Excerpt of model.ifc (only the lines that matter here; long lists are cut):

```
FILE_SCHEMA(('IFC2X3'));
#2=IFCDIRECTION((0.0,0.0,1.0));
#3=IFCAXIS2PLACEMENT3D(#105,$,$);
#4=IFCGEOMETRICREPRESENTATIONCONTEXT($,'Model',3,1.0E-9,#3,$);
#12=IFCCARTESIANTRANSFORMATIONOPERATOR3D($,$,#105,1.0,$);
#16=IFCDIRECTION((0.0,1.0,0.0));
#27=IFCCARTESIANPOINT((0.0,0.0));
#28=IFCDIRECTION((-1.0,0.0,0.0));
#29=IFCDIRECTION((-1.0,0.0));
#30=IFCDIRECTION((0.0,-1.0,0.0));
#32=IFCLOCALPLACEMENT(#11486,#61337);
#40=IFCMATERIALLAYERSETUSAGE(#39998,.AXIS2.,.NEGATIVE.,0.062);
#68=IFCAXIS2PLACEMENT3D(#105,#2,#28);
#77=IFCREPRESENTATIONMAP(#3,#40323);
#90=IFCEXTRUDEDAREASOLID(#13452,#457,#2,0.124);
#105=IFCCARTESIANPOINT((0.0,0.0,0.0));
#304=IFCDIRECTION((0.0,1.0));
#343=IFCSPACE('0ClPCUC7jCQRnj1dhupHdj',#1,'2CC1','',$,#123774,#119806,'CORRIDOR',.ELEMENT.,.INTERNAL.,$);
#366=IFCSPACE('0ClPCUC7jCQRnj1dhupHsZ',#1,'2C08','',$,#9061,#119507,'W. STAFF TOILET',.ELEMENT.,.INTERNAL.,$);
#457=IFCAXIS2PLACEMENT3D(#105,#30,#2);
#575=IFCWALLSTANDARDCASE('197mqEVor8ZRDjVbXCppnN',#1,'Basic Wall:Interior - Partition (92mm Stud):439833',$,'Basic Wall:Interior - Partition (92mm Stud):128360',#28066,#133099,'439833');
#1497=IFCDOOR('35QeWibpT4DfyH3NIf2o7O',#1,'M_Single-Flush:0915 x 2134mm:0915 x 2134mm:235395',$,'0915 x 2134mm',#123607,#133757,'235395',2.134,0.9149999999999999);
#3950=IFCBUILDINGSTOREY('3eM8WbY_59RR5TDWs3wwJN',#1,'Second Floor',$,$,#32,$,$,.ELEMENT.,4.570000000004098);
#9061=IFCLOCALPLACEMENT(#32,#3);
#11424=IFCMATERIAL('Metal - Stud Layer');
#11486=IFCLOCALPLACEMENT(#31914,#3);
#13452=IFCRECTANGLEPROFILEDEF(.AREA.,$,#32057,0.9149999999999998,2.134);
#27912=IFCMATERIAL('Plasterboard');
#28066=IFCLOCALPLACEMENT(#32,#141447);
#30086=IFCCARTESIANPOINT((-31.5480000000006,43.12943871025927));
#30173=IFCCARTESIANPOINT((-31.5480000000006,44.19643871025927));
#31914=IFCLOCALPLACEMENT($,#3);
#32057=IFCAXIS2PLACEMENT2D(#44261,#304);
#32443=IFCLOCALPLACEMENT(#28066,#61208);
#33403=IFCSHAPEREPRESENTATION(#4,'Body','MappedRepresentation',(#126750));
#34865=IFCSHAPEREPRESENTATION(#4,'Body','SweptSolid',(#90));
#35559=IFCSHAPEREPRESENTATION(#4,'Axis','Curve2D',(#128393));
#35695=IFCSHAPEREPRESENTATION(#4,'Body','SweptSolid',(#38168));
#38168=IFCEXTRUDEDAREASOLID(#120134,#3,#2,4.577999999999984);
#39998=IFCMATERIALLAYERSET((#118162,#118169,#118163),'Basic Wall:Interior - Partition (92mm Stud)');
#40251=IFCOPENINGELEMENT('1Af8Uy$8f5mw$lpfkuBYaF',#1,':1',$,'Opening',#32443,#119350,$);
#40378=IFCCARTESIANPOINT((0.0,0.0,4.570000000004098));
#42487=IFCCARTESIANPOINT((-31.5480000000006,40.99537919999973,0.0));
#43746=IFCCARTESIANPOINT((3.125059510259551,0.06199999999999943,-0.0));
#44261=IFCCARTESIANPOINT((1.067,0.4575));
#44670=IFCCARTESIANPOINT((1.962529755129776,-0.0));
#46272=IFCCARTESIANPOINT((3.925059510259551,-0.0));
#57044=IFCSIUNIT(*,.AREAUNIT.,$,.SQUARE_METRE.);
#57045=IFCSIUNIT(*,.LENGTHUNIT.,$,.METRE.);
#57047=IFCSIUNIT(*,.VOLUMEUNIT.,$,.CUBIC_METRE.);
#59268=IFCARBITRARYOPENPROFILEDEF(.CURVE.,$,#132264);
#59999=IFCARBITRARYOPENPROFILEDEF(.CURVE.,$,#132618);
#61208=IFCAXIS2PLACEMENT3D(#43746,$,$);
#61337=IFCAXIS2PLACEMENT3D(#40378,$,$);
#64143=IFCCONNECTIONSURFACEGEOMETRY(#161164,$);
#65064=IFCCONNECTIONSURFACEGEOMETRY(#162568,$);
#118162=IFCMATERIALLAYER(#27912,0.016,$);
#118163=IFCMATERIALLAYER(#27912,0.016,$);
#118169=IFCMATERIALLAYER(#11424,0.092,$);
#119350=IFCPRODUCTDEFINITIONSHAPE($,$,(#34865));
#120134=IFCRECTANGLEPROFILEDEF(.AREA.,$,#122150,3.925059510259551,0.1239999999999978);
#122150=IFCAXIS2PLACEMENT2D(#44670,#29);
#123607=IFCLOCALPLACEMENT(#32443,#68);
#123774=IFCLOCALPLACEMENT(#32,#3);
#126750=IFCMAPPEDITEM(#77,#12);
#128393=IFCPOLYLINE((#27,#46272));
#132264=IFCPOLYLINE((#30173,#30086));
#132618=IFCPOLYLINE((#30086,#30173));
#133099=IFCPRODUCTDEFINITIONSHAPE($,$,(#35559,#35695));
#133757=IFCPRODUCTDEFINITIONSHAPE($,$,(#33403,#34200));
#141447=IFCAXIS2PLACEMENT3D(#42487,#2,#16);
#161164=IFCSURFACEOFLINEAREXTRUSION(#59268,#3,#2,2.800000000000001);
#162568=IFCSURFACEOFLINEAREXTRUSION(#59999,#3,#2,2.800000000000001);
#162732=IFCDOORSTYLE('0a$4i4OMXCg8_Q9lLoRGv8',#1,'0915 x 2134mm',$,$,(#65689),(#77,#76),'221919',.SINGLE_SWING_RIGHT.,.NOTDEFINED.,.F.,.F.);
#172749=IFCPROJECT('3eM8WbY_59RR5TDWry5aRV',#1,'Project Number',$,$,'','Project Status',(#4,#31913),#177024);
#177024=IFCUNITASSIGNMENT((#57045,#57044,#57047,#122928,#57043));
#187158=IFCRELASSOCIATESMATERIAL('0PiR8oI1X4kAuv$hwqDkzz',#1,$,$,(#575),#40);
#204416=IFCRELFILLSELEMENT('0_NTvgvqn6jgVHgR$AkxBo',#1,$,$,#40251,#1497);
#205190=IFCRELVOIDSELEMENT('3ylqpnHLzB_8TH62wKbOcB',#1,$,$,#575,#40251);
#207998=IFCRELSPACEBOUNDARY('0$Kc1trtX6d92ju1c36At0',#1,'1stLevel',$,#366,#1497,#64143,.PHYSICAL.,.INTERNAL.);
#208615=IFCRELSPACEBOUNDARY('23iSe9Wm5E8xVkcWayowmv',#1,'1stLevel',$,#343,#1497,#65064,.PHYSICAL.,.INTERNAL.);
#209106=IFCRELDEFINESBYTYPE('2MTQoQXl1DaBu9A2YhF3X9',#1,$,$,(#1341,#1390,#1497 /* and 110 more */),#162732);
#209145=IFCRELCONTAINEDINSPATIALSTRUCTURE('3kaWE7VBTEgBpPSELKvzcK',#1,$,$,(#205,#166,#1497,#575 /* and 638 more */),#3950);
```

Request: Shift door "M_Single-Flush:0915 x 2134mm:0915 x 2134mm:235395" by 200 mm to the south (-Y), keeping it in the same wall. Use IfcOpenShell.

```python
import numpy as np
import ifcopenshell
import ifcopenshell.api.geometry
import ifcopenshell.util.placement
import ifcopenshell.util.unit

model = ifcopenshell.open("model.ifc")
unit_scale = ifcopenshell.util.unit.calculate_unit_scale(model)

door = model.by_guid("35QeWibpT4DfyH3NIf2o7O")
opening = door.FillsVoids[0].RelatingOpeningElement
wall = opening.VoidsElements[0].RelatingBuildingElement

wall_matrix = ifcopenshell.util.placement.get_local_placement(wall.ObjectPlacement)
shift = wall_matrix[:3, 0] * -0.2 / unit_scale
before = ifcopenshell.util.placement.get_local_placement(door.ObjectPlacement)[:3, 3].copy()

# The door is placed relative to its opening, so it follows when the opening moves.
matrix = ifcopenshell.util.placement.get_local_placement(opening.ObjectPlacement)
matrix[:3, 3] += shift
ifcopenshell.api.geometry.edit_object_placement(
    model, product=opening, matrix=matrix, is_si=False, should_transform_children=True
)

# Space boundary surfaces are stored in each space's coordinates; move them too.
for rel in door.ProvidesBoundaries:
    if not rel.ConnectionGeometry:
        continue
    surface = rel.ConnectionGeometry.SurfaceOnRelatingElement
    space_matrix = ifcopenshell.util.placement.get_local_placement(rel.RelatingSpace.ObjectPlacement)
    point = np.array(surface.Position.Location.Coordinates) + space_matrix[:3, :3].T @ shift
    surface.Position = model.createIfcAxis2Placement3D(
        model.createIfcCartesianPoint(point.tolist()), surface.Position.Axis, surface.Position.RefDirection
    )

after = ifcopenshell.util.placement.get_local_placement(door.ObjectPlacement)[:3, 3]
print("door moved by", (after - before).round(3) + 0.0)

model.write("model_edited.ifc")
```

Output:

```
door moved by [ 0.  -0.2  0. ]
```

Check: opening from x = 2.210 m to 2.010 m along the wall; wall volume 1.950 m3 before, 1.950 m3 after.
